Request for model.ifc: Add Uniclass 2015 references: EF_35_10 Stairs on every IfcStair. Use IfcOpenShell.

First a look at what the model holds.

```python
import ifcopenshell

model = ifcopenshell.open("model.ifc")
print(model.schema)
print("classifications:", [c.Name for c in model.by_type("IfcClassification")])
for ifc_class in ("IfcDoor", "IfcRoof", "IfcStair", "IfcWall", "IfcWindow"):
    print(ifc_class, len(model.by_type(ifc_class)))
```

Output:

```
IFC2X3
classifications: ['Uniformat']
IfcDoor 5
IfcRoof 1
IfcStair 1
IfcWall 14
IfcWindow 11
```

```python
import ifcopenshell
import ifcopenshell.api.classification

model = ifcopenshell.open("model.ifc")

# IFC2X3 requires Source and Edition and has no link from the project to the system.
system = model.create_entity("IfcClassification", Source="NBS", Edition="2015", Name="Uniclass 2015")

codes = {
    "IfcStair": ("EF_35_10", "Stairs"),
}
for ifc_class, (code, name) in codes.items():
    products = model.by_type(ifc_class)
    ifcopenshell.api.classification.add_reference(
        model, products=products, classification=system, identification=code, name=name
    )
    print(code, len(products))

model.write("model_edited.ifc")
```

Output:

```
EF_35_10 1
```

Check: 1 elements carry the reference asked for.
